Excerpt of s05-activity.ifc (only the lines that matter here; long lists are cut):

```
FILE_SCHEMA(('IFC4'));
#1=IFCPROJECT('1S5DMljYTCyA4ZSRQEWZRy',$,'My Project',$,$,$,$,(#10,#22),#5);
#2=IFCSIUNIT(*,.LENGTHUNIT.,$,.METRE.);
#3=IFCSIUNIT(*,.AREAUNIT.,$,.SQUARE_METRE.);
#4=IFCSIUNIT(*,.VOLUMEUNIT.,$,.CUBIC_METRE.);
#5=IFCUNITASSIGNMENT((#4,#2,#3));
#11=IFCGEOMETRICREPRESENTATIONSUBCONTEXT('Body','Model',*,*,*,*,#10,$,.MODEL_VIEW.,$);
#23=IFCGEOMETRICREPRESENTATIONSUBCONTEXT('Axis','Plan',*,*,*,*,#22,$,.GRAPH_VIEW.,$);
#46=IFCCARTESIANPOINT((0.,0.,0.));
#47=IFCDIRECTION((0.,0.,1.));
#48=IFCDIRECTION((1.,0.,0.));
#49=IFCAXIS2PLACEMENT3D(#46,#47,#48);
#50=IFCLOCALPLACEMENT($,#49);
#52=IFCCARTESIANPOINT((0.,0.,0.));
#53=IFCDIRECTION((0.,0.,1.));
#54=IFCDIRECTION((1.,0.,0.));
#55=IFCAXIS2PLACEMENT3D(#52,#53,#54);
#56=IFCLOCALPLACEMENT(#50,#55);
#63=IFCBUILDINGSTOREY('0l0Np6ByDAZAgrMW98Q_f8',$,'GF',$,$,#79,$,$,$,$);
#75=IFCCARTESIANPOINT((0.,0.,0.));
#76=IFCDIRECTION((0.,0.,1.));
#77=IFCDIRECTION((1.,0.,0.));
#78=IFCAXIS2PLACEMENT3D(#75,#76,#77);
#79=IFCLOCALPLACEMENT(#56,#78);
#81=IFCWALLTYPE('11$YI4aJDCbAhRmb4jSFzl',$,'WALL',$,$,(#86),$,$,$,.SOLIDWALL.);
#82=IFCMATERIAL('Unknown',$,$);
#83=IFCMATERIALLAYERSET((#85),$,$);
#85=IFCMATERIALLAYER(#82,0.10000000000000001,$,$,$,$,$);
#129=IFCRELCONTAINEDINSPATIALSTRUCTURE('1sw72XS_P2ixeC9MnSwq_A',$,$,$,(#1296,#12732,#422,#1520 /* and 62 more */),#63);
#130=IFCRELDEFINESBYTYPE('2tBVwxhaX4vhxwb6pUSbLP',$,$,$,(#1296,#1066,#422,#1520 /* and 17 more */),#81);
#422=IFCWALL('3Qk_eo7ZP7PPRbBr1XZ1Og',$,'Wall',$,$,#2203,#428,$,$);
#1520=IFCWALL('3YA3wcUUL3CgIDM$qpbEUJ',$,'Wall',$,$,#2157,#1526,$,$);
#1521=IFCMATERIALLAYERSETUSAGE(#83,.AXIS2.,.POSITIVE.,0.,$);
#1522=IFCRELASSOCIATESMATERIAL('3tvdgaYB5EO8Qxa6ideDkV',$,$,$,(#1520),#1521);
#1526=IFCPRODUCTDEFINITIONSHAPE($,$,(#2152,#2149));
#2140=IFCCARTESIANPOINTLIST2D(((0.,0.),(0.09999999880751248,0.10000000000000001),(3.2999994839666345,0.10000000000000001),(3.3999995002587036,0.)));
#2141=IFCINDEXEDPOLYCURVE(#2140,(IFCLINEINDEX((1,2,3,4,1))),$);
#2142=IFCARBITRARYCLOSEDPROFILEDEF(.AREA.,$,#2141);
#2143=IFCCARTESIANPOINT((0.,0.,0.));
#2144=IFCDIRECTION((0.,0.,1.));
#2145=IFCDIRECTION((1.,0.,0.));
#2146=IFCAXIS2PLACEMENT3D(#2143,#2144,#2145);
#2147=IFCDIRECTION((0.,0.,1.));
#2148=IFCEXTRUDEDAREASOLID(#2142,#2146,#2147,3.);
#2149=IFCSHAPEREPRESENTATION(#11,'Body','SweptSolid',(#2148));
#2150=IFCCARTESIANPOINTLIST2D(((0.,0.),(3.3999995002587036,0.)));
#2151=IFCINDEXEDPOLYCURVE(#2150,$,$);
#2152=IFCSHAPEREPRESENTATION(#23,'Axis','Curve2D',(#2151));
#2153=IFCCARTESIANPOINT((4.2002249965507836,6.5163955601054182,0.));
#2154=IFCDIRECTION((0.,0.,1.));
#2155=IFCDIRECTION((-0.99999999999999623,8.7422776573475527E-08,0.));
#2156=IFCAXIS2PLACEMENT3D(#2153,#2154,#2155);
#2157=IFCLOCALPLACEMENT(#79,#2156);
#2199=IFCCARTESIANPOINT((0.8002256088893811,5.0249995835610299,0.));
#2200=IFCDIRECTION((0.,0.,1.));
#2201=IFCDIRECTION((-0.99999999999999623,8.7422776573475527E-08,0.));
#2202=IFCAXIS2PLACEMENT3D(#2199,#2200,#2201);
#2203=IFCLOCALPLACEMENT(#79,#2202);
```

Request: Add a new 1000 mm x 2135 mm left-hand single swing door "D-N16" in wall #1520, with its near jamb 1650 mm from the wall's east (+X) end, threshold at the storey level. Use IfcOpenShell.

```python
import numpy as np
import ifcopenshell
import ifcopenshell.api.feature
import ifcopenshell.api.geometry
import ifcopenshell.api.root
import ifcopenshell.api.spatial
import ifcopenshell.geom
import ifcopenshell.util.element
import ifcopenshell.util.placement
import ifcopenshell.util.representation
import ifcopenshell.util.shape
import ifcopenshell.util.unit

model = ifcopenshell.open("s05-activity.ifc")
unit_scale = ifcopenshell.util.unit.calculate_unit_scale(model)
settings = ifcopenshell.geom.settings()


def volume(element):
    """Net volume in cubic metres, openings subtracted."""
    shape = ifcopenshell.geom.create_shape(settings, element)
    return ifcopenshell.util.shape.get_volume(shape.geometry)


wall = model.by_guid("3YA3wcUUL3CgIDM$qpbEUJ")
storey = ifcopenshell.util.element.get_container(wall, ifc_class="IfcBuildingStorey")
context = ifcopenshell.util.representation.get_context(model, "Model", "Body", "MODEL_VIEW")
before = volume(wall)

width, height, from_end, sill = 1, 2.135, 1.65, 0.0  # metres

# The wall runs along its own X axis, and the end named is its -X end.
wall_shape = ifcopenshell.geom.create_shape(settings, wall)
x, y, z = ifcopenshell.util.shape.get_vertices(wall_shape.geometry).T
start = x.min() + from_end
face, thickness = float(y.min()), float(y.max() - y.min())
wall_matrix = ifcopenshell.util.placement.get_local_placement(wall.ObjectPlacement)
level = ifcopenshell.util.placement.get_local_placement(storey.ObjectPlacement)[2, 3]


def in_wall(x, y):
    """Placement at x, y metres in the wall's axes, at sill height."""
    matrix = wall_matrix.copy()
    matrix[:, 3] = wall_matrix @ np.array([x / unit_scale, y / unit_scale, 0.0, 1.0])
    matrix[2, 3] = level + sill / unit_scale
    return matrix


# Opening: a box that overshoots both wall faces by 50 mm.
opening = ifcopenshell.api.root.create_entity(model, ifc_class="IfcOpeningElement", predefined_type="OPENING")
box = ifcopenshell.api.geometry.add_wall_representation(
    model, context=context, length=width, height=height, thickness=thickness + 0.1
)
ifcopenshell.api.geometry.assign_representation(model, product=opening, representation=box)
ifcopenshell.api.geometry.edit_object_placement(model, product=opening, matrix=in_wall(start, face - 0.05), is_si=False)
ifcopenshell.api.feature.add_feature(model, feature=opening, element=wall)

door = ifcopenshell.api.root.create_entity(model, ifc_class="IfcDoor", name="D-N16", predefined_type="DOOR")
door.OverallWidth, door.OverallHeight = width / unit_scale, height / unit_scale
door.OperationType = "SINGLE_SWING_LEFT"
body = ifcopenshell.api.geometry.add_door_representation(
    model,
    context=context,
    overall_width=door.OverallWidth,
    overall_height=door.OverallHeight,
    operation_type="SINGLE_SWING_LEFT",
    lining_properties={"LiningDepth": thickness / unit_scale, "ThresholdDepth": thickness / unit_scale},
)
ifcopenshell.api.geometry.assign_representation(model, product=door, representation=body)
ifcopenshell.api.spatial.assign_container(model, products=[door], relating_structure=storey)
ifcopenshell.api.feature.add_filling(model, opening=opening, element=door)

# The lining spans the wall, so the door starts at the wall face.
ifcopenshell.api.geometry.edit_object_placement(model, product=door, matrix=in_wall(start, face), is_si=False)

after = volume(wall)

print(f"wall volume {before:.3f} -> {after:.3f} m3")

model.write("s05-activity_updated.ifc")
```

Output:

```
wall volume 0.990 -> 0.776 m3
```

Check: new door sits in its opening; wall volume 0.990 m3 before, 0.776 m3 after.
